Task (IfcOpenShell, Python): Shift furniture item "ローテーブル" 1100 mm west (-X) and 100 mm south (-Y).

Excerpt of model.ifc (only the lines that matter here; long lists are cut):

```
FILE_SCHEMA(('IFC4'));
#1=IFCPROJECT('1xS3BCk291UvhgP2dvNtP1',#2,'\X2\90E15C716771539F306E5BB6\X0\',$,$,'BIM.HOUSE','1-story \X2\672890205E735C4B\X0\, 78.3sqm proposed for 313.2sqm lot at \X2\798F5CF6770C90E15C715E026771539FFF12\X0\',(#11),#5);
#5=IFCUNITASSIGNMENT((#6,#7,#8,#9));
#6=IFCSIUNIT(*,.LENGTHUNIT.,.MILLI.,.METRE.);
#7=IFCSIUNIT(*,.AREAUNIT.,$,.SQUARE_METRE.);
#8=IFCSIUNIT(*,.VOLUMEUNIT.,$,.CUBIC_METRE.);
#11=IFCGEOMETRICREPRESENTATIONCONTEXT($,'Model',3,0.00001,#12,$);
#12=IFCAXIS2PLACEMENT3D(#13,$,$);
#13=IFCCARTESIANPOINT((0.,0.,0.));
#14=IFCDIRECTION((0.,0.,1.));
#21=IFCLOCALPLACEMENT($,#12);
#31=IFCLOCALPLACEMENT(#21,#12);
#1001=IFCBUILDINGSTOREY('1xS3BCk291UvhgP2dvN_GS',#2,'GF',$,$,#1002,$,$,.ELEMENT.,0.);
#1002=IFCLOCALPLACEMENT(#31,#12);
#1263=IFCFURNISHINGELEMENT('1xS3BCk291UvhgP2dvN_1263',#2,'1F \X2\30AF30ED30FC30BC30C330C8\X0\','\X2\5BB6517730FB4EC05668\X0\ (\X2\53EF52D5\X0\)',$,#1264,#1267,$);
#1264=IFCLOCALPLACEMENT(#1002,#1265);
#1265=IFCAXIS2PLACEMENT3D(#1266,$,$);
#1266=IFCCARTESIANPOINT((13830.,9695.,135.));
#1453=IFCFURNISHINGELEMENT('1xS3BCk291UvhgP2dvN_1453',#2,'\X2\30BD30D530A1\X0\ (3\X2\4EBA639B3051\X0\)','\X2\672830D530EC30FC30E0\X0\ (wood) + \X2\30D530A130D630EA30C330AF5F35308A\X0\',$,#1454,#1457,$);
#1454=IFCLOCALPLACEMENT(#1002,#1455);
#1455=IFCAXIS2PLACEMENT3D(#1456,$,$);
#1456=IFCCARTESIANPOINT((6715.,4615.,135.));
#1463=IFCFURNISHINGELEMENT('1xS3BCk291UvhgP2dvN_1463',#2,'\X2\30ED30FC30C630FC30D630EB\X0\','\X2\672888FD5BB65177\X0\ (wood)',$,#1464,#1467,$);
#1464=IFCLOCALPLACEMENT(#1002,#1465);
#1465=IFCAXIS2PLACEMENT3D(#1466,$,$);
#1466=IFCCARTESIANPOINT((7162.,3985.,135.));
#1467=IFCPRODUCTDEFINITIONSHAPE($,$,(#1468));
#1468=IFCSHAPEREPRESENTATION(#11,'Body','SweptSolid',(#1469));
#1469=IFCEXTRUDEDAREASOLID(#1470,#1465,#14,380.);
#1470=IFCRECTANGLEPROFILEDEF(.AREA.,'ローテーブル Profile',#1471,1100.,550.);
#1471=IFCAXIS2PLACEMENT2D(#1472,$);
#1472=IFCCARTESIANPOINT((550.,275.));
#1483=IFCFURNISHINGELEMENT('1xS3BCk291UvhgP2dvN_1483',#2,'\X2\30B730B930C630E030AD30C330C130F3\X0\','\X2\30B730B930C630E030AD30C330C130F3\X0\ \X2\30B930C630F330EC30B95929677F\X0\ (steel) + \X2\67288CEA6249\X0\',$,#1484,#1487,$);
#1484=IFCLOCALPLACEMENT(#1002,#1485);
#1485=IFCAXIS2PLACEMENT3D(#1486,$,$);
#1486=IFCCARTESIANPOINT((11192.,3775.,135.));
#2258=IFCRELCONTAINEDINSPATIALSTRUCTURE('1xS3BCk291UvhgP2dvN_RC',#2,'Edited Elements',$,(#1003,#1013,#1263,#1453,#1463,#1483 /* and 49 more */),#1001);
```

```python
import ifcopenshell
import ifcopenshell.api.geometry
import ifcopenshell.util.placement
import ifcopenshell.util.unit

model = ifcopenshell.open("model.ifc")
unit_scale = ifcopenshell.util.unit.calculate_unit_scale(model)

item = model.by_guid("1xS3BCk291UvhgP2dvN_1463")
matrix = ifcopenshell.util.placement.get_local_placement(item.ObjectPlacement)
matrix[0, 3] -= 1.1 / unit_scale
matrix[1, 3] -= 0.1 / unit_scale
ifcopenshell.api.geometry.edit_object_placement(model, product=item, matrix=matrix, is_si=False)

print(ifcopenshell.util.placement.get_local_placement(item.ObjectPlacement).round(3) + 0.0)

model.write("model_v2.ifc")
```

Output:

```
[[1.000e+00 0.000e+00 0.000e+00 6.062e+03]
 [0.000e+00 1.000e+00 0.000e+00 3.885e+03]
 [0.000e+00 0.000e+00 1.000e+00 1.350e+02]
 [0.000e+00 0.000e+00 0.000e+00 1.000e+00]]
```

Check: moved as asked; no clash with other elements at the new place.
